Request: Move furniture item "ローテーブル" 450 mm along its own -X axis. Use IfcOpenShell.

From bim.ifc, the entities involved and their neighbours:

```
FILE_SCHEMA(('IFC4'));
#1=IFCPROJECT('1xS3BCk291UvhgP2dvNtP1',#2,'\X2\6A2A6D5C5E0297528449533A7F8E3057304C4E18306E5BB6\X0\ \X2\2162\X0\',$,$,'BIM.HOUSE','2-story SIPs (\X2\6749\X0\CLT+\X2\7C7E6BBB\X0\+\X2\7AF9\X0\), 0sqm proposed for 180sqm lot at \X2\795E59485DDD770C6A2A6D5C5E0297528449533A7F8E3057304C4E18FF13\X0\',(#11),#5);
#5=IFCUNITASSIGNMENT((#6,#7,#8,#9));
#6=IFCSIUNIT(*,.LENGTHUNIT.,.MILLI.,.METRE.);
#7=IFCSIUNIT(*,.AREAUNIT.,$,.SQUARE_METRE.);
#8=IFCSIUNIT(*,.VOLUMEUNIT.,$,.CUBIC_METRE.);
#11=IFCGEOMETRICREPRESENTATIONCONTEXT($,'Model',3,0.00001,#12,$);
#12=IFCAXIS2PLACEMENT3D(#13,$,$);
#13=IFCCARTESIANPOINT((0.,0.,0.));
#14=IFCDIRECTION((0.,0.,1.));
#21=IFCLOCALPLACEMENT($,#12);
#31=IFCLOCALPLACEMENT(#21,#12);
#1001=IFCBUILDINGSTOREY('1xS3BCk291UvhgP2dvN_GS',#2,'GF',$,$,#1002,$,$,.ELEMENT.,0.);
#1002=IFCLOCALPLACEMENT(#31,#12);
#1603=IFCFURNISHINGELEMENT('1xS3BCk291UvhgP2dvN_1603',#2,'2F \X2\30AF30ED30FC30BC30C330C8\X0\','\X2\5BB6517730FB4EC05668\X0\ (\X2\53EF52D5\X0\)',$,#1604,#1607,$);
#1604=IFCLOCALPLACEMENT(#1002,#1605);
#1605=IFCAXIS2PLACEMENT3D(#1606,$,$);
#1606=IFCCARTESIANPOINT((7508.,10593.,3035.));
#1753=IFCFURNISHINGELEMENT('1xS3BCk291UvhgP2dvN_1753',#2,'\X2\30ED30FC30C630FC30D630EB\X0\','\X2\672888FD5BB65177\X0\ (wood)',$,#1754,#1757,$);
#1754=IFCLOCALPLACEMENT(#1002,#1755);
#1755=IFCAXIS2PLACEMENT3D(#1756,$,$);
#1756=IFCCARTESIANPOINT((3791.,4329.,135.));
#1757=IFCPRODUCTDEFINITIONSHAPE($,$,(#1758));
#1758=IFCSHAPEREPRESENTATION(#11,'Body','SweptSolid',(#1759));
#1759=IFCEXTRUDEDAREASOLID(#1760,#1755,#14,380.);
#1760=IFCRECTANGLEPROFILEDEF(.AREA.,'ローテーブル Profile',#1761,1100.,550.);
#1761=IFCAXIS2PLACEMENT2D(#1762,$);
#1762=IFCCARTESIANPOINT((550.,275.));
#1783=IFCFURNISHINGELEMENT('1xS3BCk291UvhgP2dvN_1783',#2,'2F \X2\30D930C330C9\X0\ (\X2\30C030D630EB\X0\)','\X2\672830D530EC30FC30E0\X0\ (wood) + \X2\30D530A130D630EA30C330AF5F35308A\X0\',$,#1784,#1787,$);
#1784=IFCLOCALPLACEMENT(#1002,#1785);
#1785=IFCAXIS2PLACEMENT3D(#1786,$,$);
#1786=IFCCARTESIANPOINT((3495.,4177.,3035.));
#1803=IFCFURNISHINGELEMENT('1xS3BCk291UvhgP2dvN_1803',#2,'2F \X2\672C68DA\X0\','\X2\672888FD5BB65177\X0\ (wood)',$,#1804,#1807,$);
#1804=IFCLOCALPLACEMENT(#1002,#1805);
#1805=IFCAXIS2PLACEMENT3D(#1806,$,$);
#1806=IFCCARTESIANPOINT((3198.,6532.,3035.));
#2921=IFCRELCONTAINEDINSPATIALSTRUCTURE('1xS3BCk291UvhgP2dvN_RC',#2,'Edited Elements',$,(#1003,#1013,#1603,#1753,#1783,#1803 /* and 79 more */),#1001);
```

```python
import ifcopenshell
import ifcopenshell.api.geometry
import ifcopenshell.util.placement
import ifcopenshell.util.unit

model = ifcopenshell.open("bim.ifc")
unit_scale = ifcopenshell.util.unit.calculate_unit_scale(model)

item = model.by_guid("1xS3BCk291UvhgP2dvN_1753")
matrix = ifcopenshell.util.placement.get_local_placement(item.ObjectPlacement)
matrix[:3, 3] -= matrix[:3, 0] * 0.45 / unit_scale
ifcopenshell.api.geometry.edit_object_placement(model, product=item, matrix=matrix, is_si=False)

print(ifcopenshell.util.placement.get_local_placement(item.ObjectPlacement).round(3) + 0.0)

model.write("bim_updated.ifc")
```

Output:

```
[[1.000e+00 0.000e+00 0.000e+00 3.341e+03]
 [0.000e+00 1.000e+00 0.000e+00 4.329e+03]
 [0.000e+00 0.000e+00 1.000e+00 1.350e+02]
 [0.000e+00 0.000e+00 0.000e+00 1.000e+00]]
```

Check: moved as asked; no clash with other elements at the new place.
